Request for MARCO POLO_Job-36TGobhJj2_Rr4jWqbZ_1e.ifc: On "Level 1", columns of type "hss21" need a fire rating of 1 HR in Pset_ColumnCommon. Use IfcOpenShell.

First a look at what the model holds.

```python
import ifcopenshell
import ifcopenshell.util.element

model = ifcopenshell.open("MARCO POLO_Job-36TGobhJj2_Rr4jWqbZ_1e.ifc")
print(model.schema)
storey = next(s for s in model.by_type("IfcBuildingStorey") if s.Name == "Level 1")
columns = [e for e in ifcopenshell.util.element.get_decomposition(storey) if e.is_a("IfcColumn")]
seen = {}
for e in columns:
    element_type = ifcopenshell.util.element.get_type(e)
    key = (element_type.Name if element_type != e and element_type else None, ifcopenshell.util.element.get_pset(e, "Pset_ColumnCommon", "FireRating"))
    seen[key] = seen.get(key, 0) + 1
for (name, value), count in sorted(seen.items(), key=str):
    print(count, "x", name, "|", value)
```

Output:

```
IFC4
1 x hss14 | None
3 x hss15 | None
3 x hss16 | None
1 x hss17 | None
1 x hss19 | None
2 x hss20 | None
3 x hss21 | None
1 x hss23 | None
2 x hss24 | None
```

```python
import ifcopenshell
import ifcopenshell.api.pset
import ifcopenshell.util.element

model = ifcopenshell.open("MARCO POLO_Job-36TGobhJj2_Rr4jWqbZ_1e.ifc")

storey = next(s for s in model.by_type("IfcBuildingStorey") if s.Name == "Level 1")
columns = [e for e in ifcopenshell.util.element.get_decomposition(storey) if e.is_a("IfcColumn")]

count = 0
for e in columns:
    element_type = ifcopenshell.util.element.get_type(e)
    if element_type in (None, e) or element_type.Name != "hss21":
        continue
    # add_pset returns the element's existing set when there is one.
    pset = ifcopenshell.api.pset.add_pset(model, product=e, name="Pset_ColumnCommon")
    ifcopenshell.api.pset.edit_pset(model, pset=pset, properties={"FireRating": "1 HR"})
    count += 1

print(count, "columns updated")

model.write("MARCO POLO_Job-36TGobhJj2_Rr4jWqbZ_1e_v2.ifc")
```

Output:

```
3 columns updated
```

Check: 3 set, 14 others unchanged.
